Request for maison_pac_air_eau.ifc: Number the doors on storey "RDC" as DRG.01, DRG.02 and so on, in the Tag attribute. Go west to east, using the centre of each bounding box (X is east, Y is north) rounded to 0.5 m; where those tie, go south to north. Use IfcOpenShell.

First a look at what the model holds.

```python
import ifcopenshell
import ifcopenshell.util.element
import ifcopenshell.util.placement

model = ifcopenshell.open("maison_pac_air_eau.ifc")
print(model.schema)
storey = next(s for s in model.by_type("IfcBuildingStorey") if s.Name == "RDC")
doors = [e for e in ifcopenshell.util.element.get_decomposition(storey) if e.is_a("IfcDoor")]
for e in sorted(doors, key=lambda e: e.id()):
    origin = ifcopenshell.util.placement.get_local_placement(e.ObjectPlacement)[:3, 3]
    print(e.id(), e.Tag, e.Name, origin.round(2) + 0.0, sep=" | ")
```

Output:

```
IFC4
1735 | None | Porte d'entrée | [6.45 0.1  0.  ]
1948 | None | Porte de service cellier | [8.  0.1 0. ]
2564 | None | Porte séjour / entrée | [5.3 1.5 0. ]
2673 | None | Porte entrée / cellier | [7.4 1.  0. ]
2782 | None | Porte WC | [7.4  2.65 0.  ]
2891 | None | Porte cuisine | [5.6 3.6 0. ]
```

```python
import ifcopenshell
import ifcopenshell.geom
import ifcopenshell.util.element
import ifcopenshell.util.shape

model = ifcopenshell.open("maison_pac_air_eau.ifc")
settings = ifcopenshell.geom.settings()
settings.set("use-world-coords", True)


def centre(element):
    shape = ifcopenshell.geom.create_shape(settings, element)
    return ifcopenshell.util.shape.get_bbox_centroid(shape.geometry)


storey = next(s for s in model.by_type("IfcBuildingStorey") if s.Name == "RDC")
doors = [e for e in ifcopenshell.util.element.get_decomposition(storey) if e.is_a("IfcDoor")]

# Insertion points can sit at a corner or the storey origin, so sort by the geometry (in metres).
centres = {e: centre(e) for e in doors}
doors.sort(key=lambda e: (round(centres[e][0] / 0.5), centres[e][1]))

for i, e in enumerate(doors, start=1):
    number = f"DRG.{i:02d}"
    e.Tag = number
    print(e.id(), number)

model.write("maison_pac_air_eau_rev.ifc")
```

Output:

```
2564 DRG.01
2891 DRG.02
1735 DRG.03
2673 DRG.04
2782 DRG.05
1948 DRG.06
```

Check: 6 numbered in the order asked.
